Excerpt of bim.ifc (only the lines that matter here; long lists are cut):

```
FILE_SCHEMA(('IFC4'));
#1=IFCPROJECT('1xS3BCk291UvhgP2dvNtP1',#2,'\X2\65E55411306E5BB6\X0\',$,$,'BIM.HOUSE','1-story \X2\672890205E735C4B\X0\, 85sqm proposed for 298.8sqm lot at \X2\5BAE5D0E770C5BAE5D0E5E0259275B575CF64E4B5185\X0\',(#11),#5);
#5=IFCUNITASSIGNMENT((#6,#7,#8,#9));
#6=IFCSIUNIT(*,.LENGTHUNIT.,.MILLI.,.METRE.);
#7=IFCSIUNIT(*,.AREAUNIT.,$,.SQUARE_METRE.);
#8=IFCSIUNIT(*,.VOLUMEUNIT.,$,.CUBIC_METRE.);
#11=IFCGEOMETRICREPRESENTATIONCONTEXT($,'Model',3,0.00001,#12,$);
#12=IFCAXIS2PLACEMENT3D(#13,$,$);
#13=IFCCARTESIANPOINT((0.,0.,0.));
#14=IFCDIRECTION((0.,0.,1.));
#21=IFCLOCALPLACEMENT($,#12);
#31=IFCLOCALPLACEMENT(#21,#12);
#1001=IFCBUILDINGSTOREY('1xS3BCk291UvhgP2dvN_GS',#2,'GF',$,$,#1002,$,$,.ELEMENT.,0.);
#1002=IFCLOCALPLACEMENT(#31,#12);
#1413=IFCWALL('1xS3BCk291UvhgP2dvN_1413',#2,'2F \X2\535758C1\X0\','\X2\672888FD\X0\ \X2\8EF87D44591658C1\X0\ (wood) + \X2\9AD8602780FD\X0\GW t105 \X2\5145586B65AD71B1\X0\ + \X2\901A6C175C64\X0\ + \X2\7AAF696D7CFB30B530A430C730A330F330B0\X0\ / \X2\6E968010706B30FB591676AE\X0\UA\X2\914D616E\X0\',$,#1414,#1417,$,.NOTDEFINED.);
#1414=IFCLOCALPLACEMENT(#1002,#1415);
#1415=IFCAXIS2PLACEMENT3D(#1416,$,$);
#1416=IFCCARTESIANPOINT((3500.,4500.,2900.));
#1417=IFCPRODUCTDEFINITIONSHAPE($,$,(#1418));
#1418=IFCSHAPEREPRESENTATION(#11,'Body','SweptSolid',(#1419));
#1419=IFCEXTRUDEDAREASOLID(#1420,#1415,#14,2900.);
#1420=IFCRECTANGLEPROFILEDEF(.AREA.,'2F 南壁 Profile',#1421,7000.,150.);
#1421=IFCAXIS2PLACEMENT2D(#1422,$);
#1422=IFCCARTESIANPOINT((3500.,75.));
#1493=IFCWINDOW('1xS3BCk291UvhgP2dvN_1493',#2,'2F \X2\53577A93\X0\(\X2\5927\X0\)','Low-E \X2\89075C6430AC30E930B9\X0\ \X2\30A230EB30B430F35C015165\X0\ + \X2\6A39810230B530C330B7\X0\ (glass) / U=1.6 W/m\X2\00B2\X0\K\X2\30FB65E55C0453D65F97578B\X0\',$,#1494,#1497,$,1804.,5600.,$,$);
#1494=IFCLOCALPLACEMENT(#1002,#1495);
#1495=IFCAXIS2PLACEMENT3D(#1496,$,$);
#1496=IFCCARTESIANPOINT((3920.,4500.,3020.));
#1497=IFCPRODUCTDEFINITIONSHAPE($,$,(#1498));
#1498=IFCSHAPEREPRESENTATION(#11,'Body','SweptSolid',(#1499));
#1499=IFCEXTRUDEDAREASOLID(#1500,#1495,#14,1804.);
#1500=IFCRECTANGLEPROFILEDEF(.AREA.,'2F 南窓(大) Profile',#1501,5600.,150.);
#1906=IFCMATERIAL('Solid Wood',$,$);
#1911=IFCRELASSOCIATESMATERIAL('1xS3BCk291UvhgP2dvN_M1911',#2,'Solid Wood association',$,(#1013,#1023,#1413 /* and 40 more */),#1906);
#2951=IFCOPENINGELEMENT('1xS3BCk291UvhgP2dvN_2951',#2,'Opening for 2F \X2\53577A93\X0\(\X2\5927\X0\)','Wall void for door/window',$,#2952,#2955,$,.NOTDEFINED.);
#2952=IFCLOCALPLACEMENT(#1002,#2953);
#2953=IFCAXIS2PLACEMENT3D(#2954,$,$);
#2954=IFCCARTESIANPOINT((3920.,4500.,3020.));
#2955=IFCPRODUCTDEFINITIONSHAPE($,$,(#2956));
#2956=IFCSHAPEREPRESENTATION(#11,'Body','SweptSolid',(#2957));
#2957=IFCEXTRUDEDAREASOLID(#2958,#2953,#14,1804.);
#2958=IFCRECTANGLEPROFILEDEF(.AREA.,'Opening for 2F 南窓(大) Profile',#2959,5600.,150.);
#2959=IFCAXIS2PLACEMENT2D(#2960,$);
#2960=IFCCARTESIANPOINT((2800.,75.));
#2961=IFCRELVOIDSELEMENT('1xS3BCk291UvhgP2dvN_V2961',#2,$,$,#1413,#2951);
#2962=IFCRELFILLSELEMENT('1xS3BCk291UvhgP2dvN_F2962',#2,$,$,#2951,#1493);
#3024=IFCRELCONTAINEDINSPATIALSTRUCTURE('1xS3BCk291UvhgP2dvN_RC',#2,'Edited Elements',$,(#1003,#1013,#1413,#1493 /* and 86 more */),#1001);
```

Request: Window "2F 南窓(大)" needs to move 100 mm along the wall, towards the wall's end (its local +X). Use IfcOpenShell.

```python
import ifcopenshell
import ifcopenshell.api.geometry
import ifcopenshell.util.placement

model = ifcopenshell.open("bim.ifc")

window = model.by_guid("1xS3BCk291UvhgP2dvN_1493")
opening = window.FillsVoids[0].RelatingOpeningElement
wall = opening.VoidsElements[0].RelatingBuildingElement

wall_matrix = ifcopenshell.util.placement.get_local_placement(wall.ObjectPlacement)
shift = wall_matrix[:3, 0] * 100.0
before = ifcopenshell.util.placement.get_local_placement(window.ObjectPlacement)[:3, 3].copy()

# The window is not placed relative to its opening, so move both.
for product in (opening, window):
    matrix = ifcopenshell.util.placement.get_local_placement(product.ObjectPlacement)
    matrix[:3, 3] += shift
    ifcopenshell.api.geometry.edit_object_placement(model, product=product, matrix=matrix, is_si=False)

after = ifcopenshell.util.placement.get_local_placement(window.ObjectPlacement)[:3, 3]
print("window moved by", (after - before).round(3) + 0.0)

model.write("bim_edited.ifc")
```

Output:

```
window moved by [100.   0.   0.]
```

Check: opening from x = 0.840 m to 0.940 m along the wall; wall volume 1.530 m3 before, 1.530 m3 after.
